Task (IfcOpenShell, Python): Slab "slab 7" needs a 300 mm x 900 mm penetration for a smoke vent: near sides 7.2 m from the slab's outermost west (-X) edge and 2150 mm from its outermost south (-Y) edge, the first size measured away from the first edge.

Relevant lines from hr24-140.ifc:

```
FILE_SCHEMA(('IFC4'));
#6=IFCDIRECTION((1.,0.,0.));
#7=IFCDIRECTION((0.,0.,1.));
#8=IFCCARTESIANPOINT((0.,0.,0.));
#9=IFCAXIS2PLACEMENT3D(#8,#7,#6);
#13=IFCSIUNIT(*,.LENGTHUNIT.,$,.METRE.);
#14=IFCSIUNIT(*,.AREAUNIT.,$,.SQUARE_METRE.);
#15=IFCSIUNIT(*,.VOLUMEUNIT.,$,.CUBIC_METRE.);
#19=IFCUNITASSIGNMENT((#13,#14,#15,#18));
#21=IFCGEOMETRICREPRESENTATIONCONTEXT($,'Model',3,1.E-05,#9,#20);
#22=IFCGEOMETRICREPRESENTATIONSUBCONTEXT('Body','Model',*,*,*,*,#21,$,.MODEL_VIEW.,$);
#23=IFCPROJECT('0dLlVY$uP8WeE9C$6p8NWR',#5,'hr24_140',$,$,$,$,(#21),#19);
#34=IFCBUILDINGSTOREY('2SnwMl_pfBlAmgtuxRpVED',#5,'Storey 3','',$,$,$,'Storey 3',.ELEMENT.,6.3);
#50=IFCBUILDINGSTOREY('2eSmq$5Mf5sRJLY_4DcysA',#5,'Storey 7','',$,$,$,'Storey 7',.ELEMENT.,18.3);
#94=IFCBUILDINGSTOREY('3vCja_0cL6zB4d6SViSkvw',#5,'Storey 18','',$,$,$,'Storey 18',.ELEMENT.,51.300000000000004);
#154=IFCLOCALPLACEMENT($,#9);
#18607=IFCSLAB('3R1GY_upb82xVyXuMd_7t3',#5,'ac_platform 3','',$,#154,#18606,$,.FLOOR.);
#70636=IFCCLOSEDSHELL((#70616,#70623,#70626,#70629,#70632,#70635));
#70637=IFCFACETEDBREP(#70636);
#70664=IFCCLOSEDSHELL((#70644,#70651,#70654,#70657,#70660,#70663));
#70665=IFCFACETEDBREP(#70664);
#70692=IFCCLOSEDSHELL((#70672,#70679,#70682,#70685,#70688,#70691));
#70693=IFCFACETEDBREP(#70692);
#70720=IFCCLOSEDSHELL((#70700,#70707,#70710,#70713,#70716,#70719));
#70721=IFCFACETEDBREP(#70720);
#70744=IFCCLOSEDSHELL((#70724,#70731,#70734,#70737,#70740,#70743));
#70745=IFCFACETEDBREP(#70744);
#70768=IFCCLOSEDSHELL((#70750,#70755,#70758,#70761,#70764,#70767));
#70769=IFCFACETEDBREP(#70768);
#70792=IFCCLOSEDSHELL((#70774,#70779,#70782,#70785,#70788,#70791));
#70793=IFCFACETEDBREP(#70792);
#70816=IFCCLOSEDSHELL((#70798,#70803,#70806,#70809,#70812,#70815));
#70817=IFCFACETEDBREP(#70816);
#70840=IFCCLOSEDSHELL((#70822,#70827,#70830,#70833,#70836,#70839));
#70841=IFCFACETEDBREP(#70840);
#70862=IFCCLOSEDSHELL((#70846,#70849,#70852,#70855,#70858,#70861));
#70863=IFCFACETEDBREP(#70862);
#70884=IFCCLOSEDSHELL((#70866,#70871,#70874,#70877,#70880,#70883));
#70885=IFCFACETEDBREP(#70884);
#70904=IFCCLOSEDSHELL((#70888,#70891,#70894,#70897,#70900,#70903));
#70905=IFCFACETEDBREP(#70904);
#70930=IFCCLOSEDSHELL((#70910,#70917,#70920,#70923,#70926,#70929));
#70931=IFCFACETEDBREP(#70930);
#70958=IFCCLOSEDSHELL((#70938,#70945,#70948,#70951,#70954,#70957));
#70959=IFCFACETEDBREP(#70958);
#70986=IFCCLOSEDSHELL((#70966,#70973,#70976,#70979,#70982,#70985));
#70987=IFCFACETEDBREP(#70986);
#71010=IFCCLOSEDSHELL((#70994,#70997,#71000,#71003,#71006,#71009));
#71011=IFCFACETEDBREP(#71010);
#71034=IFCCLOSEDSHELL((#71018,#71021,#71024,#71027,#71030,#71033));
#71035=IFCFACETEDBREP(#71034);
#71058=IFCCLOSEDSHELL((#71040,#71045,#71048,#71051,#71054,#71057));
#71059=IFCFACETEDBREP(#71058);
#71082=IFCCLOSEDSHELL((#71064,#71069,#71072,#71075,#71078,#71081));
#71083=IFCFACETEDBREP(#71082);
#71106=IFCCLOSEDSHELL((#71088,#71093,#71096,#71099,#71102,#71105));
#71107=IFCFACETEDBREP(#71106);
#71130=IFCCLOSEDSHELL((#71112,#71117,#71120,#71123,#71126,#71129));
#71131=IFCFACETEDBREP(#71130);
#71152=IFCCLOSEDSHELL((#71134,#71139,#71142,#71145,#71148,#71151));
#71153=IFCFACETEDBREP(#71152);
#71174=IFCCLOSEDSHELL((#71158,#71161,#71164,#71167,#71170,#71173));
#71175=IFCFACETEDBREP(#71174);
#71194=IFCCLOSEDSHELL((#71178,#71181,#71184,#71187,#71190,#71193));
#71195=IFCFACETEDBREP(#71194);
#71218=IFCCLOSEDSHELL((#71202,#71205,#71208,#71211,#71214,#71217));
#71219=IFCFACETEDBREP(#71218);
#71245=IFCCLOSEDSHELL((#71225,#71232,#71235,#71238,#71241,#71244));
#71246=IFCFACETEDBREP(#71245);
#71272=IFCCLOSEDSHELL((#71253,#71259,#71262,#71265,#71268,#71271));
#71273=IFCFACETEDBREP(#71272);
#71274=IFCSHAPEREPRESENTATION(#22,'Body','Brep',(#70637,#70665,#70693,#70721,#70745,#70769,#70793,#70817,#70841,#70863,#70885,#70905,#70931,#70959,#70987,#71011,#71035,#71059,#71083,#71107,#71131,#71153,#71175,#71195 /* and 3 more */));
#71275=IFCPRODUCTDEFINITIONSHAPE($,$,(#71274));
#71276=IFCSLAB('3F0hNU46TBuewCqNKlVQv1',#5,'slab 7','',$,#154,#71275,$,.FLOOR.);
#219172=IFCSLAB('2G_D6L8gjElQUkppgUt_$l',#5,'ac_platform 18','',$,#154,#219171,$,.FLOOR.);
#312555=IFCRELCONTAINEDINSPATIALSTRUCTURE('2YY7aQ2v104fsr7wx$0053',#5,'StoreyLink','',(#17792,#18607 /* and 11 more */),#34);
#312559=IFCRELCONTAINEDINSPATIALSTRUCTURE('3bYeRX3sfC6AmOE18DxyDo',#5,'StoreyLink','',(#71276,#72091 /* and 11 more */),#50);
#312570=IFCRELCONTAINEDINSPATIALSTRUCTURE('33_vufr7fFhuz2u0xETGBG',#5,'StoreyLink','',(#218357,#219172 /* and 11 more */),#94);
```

```python
import numpy as np
import ifcopenshell
import ifcopenshell.api.feature
import ifcopenshell.api.geometry
import ifcopenshell.api.root
import ifcopenshell.geom
import ifcopenshell.util.placement
import ifcopenshell.util.representation
import ifcopenshell.util.shape
import ifcopenshell.util.unit

model = ifcopenshell.open("hr24-140.ifc")
unit_scale = ifcopenshell.util.unit.calculate_unit_scale(model)
settings = ifcopenshell.geom.settings()


def volume(element):
    """Net volume in cubic metres, openings subtracted."""
    shape = ifcopenshell.geom.create_shape(settings, element)
    return ifcopenshell.util.shape.get_volume(shape.geometry)


slab = model.by_guid("3F0hNU46TBuewCqNKlVQv1")
before = volume(slab)

# Extent in the slab's own axes, in metres. The edges named are its -X and -Y sides.
slab_shape = ifcopenshell.geom.create_shape(settings, slab)
vertices = ifcopenshell.util.shape.get_vertices(slab_shape.geometry)
x_min, y_min, bottom = vertices.min(axis=0)
top = vertices[:, 2].max()

opening = ifcopenshell.api.root.create_entity(model, ifc_class="IfcOpeningElement", name="Smoke vent opening", predefined_type="OPENING")
context = ifcopenshell.util.representation.get_context(model, "Model", "Body", "MODEL_VIEW")
width, depth = 0.3, 0.9
outline = [(0.0, 0.0), (width, 0.0), (width, depth), (0.0, depth), (0.0, 0.0)]
# Overshoot both faces by 50 mm so the cut is clean.
shape = ifcopenshell.api.geometry.add_slab_representation(
    model, context=context, depth=top - bottom + 0.1, polyline=outline
)
ifcopenshell.api.geometry.assign_representation(model, product=opening, representation=shape)

matrix = ifcopenshell.util.placement.get_local_placement(slab.ObjectPlacement)
matrix[:, 3] = matrix @ np.append(np.array([x_min + 7.2, y_min + 2.15, bottom - 0.05]) / unit_scale, 1.0)
ifcopenshell.api.geometry.edit_object_placement(model, product=opening, matrix=matrix, is_si=False)
ifcopenshell.api.feature.add_feature(model, feature=opening, element=slab)

after = volume(slab)

print(f"slab volume {before:.3f} -> {after:.3f} m3")

model.write("hr24-140-out.ifc")
```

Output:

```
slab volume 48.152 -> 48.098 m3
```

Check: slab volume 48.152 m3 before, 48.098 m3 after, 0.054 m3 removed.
